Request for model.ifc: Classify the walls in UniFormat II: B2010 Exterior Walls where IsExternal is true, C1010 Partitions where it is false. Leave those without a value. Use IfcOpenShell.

First a look at what the model holds.

```python
import ifcopenshell
import ifcopenshell.util.element

model = ifcopenshell.open("model.ifc")
print(model.schema)
print("classifications:", [c.Name for c in model.by_type("IfcClassification")])
values = [ifcopenshell.util.element.get_pset(e, "Pset_WallCommon", "IsExternal") for e in model.by_type("IfcWall")]
for value in (True, False, None):
    print("IsExternal", value, values.count(value))
```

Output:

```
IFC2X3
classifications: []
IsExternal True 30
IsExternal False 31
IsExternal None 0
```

```python
import ifcopenshell
import ifcopenshell.api.classification
import ifcopenshell.util.element

model = ifcopenshell.open("model.ifc")

# IFC2X3 requires Source and Edition and has no link from the project to the system.
system = model.create_entity("IfcClassification", Source="ASTM", Edition="E1557", Name="UniFormat II")

walls = model.by_type("IfcWall")
external = {e: ifcopenshell.util.element.get_pset(e, "Pset_WallCommon", "IsExternal") for e in walls}
for flag, code, name in ((True, "B2010", "Exterior Walls"), (False, "C1010", "Partitions")):
    products = [e for e in walls if external[e] is flag]
    ifcopenshell.api.classification.add_reference(
        model, products=products, classification=system, identification=code, name=name
    )
    print(code, len(products))

model.write("model_edited.ifc")
```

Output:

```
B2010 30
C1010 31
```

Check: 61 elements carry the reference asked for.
